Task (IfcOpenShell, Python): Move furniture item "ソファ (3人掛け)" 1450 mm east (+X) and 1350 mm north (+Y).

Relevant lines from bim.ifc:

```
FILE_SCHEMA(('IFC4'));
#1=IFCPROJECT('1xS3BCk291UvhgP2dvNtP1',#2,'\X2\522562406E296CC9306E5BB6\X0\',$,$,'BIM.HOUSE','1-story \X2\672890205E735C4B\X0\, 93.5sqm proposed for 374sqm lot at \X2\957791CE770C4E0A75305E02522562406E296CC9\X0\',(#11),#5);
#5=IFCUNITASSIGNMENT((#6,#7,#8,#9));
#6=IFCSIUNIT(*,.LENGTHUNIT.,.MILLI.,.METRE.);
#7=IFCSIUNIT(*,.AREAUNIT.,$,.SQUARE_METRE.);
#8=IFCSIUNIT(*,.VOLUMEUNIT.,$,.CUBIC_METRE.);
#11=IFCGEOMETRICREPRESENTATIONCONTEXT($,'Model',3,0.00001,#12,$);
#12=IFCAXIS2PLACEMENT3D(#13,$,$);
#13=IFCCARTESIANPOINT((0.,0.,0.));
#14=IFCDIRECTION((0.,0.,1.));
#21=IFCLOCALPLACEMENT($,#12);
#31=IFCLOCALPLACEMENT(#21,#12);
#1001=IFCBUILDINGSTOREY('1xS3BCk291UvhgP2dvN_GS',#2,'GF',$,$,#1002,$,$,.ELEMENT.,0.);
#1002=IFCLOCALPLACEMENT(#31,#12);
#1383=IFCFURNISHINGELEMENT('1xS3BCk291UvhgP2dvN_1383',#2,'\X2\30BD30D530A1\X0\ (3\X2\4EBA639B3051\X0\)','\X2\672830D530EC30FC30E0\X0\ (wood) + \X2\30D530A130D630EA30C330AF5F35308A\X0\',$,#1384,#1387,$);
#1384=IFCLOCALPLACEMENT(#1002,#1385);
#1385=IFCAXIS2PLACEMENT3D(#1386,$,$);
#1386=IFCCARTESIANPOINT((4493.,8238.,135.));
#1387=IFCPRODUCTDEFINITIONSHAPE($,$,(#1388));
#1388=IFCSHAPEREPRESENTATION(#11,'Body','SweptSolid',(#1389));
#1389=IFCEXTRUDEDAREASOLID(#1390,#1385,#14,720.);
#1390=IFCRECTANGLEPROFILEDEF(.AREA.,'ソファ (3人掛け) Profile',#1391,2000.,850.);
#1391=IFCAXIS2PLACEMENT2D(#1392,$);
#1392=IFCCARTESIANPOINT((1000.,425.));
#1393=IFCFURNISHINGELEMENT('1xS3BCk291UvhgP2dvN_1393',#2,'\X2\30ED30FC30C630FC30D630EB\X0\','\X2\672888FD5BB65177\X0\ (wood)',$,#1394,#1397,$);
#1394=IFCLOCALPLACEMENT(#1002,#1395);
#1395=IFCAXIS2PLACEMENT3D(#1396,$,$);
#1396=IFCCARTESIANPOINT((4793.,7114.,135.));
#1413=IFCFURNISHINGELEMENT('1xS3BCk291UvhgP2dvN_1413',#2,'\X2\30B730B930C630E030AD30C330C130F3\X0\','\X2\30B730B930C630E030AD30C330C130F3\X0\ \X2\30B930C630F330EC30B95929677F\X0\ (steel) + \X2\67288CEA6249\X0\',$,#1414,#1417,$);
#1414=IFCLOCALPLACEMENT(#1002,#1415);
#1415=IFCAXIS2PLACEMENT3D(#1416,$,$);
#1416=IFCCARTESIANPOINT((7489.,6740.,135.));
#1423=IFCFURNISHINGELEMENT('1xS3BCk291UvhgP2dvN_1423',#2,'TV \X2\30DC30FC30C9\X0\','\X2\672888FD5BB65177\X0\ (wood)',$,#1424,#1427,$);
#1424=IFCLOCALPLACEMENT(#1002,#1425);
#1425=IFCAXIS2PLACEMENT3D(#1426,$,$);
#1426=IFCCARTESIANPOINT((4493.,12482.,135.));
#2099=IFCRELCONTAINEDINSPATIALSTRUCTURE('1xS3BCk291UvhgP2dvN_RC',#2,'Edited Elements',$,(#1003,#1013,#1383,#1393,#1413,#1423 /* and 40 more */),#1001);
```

```python
import ifcopenshell
import ifcopenshell.api.geometry
import ifcopenshell.util.placement
import ifcopenshell.util.unit

model = ifcopenshell.open("bim.ifc")
unit_scale = ifcopenshell.util.unit.calculate_unit_scale(model)

item = model.by_guid("1xS3BCk291UvhgP2dvN_1383")
matrix = ifcopenshell.util.placement.get_local_placement(item.ObjectPlacement)
matrix[0, 3] += 1.45 / unit_scale
matrix[1, 3] += 1.35 / unit_scale
ifcopenshell.api.geometry.edit_object_placement(model, product=item, matrix=matrix, is_si=False)

print(ifcopenshell.util.placement.get_local_placement(item.ObjectPlacement).round(3) + 0.0)

model.write("bim-out.ifc")
```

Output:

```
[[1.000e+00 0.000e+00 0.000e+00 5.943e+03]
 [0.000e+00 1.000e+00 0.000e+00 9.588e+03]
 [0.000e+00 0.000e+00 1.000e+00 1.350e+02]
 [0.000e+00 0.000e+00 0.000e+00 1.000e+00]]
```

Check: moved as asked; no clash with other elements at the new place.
